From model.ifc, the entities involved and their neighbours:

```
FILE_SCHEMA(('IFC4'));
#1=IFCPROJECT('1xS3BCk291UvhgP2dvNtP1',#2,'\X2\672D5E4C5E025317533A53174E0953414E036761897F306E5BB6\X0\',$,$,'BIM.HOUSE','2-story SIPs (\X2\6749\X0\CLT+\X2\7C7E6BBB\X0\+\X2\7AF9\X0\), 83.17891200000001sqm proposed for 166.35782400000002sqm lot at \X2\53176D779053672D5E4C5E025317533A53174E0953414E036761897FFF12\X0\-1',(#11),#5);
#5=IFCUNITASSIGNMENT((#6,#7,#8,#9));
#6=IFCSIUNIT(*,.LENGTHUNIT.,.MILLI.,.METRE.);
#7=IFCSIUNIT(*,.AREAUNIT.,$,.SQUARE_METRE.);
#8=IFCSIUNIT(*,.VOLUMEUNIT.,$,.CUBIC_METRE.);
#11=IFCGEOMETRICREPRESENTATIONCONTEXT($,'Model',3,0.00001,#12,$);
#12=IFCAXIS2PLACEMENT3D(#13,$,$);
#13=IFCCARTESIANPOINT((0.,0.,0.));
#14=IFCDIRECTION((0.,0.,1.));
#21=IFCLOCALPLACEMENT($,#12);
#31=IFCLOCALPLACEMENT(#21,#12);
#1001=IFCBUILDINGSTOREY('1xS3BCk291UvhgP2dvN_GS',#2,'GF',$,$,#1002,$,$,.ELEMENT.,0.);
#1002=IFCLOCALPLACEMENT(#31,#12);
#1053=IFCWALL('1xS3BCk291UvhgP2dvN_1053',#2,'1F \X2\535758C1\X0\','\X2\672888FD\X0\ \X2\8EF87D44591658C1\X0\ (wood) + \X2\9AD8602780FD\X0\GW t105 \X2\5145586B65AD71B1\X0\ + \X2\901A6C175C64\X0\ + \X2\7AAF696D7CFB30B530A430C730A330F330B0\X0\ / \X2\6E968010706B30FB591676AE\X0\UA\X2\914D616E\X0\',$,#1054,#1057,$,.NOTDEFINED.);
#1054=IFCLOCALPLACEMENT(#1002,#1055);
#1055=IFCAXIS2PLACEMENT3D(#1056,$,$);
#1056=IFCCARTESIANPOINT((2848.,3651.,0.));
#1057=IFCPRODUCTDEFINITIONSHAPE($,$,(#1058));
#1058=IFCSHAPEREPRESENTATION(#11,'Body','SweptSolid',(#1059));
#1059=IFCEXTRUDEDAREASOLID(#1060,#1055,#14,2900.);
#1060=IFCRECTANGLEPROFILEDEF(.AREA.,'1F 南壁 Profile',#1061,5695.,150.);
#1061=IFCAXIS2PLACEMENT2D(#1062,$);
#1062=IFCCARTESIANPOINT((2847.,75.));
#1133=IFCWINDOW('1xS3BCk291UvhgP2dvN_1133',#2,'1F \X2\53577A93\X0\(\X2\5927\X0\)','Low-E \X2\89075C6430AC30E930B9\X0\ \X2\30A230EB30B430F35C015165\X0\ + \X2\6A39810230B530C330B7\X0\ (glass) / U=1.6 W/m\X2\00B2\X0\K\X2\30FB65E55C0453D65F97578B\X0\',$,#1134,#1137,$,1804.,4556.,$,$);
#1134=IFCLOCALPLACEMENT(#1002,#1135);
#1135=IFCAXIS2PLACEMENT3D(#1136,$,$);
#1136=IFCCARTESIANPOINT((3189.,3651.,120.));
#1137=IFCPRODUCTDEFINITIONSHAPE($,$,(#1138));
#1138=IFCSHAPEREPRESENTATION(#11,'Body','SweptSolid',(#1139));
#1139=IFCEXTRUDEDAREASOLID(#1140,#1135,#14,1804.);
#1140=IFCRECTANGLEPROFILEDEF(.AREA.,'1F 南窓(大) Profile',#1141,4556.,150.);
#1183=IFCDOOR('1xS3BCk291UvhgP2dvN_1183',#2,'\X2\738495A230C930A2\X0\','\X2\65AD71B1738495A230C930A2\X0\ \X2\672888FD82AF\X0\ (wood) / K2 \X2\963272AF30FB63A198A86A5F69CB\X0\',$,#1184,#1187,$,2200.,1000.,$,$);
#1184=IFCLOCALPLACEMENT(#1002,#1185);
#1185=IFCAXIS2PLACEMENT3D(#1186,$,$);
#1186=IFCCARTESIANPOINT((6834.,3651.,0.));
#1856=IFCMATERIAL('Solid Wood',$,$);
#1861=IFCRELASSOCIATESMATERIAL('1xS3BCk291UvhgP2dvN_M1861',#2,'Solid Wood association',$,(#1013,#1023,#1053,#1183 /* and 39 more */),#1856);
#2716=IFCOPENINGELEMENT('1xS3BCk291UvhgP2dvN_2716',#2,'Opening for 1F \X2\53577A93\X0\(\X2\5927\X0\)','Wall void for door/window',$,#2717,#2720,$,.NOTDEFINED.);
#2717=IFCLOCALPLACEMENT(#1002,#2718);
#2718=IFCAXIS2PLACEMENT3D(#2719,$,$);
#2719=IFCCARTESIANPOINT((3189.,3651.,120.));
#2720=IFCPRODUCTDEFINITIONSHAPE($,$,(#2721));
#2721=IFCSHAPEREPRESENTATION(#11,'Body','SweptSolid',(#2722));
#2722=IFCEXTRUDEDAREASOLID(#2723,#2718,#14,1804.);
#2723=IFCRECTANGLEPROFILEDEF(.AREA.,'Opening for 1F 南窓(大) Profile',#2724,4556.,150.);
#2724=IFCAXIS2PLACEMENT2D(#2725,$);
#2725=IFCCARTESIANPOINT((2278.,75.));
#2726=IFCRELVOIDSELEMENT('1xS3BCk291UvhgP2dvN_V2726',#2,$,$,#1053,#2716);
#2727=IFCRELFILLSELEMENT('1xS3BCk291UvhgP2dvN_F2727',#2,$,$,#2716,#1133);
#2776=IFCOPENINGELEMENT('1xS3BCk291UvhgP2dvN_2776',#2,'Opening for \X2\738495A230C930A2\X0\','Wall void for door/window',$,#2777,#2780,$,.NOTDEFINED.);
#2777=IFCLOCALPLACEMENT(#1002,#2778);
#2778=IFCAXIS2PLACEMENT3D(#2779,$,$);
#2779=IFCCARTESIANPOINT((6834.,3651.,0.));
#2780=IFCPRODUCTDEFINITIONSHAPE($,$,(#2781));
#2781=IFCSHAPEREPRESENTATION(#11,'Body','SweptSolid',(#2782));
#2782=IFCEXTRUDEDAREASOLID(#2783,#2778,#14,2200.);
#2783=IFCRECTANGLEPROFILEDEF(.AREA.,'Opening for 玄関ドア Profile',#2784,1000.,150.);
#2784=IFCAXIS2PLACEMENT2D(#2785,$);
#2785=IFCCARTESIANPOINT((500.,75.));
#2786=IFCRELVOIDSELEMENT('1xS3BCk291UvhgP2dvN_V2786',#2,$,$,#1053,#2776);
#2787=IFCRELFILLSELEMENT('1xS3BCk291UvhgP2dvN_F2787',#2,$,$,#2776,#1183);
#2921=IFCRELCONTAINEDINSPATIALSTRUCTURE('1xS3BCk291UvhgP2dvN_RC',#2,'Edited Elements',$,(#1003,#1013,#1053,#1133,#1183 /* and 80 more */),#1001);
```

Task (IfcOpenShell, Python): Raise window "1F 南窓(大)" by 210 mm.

```python
import numpy as np
import ifcopenshell
import ifcopenshell.api.geometry
import ifcopenshell.util.placement
import ifcopenshell.util.unit

model = ifcopenshell.open("model.ifc")
unit_scale = ifcopenshell.util.unit.calculate_unit_scale(model)

window = model.by_guid("1xS3BCk291UvhgP2dvN_1133")
opening = window.FillsVoids[0].RelatingOpeningElement
dz = 0.21 / unit_scale

shift = np.array([0.0, 0.0, dz])
# The window is not placed relative to its opening, so move both.
for product in (opening, window):
    matrix = ifcopenshell.util.placement.get_local_placement(product.ObjectPlacement)
    matrix[:3, 3] += shift
    ifcopenshell.api.geometry.edit_object_placement(model, product=product, matrix=matrix, is_si=False)

print(f"moved by {dz * unit_scale:+.3f} m")

model.write("model_edited.ifc")
```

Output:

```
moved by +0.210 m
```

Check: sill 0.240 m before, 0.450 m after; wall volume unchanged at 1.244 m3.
